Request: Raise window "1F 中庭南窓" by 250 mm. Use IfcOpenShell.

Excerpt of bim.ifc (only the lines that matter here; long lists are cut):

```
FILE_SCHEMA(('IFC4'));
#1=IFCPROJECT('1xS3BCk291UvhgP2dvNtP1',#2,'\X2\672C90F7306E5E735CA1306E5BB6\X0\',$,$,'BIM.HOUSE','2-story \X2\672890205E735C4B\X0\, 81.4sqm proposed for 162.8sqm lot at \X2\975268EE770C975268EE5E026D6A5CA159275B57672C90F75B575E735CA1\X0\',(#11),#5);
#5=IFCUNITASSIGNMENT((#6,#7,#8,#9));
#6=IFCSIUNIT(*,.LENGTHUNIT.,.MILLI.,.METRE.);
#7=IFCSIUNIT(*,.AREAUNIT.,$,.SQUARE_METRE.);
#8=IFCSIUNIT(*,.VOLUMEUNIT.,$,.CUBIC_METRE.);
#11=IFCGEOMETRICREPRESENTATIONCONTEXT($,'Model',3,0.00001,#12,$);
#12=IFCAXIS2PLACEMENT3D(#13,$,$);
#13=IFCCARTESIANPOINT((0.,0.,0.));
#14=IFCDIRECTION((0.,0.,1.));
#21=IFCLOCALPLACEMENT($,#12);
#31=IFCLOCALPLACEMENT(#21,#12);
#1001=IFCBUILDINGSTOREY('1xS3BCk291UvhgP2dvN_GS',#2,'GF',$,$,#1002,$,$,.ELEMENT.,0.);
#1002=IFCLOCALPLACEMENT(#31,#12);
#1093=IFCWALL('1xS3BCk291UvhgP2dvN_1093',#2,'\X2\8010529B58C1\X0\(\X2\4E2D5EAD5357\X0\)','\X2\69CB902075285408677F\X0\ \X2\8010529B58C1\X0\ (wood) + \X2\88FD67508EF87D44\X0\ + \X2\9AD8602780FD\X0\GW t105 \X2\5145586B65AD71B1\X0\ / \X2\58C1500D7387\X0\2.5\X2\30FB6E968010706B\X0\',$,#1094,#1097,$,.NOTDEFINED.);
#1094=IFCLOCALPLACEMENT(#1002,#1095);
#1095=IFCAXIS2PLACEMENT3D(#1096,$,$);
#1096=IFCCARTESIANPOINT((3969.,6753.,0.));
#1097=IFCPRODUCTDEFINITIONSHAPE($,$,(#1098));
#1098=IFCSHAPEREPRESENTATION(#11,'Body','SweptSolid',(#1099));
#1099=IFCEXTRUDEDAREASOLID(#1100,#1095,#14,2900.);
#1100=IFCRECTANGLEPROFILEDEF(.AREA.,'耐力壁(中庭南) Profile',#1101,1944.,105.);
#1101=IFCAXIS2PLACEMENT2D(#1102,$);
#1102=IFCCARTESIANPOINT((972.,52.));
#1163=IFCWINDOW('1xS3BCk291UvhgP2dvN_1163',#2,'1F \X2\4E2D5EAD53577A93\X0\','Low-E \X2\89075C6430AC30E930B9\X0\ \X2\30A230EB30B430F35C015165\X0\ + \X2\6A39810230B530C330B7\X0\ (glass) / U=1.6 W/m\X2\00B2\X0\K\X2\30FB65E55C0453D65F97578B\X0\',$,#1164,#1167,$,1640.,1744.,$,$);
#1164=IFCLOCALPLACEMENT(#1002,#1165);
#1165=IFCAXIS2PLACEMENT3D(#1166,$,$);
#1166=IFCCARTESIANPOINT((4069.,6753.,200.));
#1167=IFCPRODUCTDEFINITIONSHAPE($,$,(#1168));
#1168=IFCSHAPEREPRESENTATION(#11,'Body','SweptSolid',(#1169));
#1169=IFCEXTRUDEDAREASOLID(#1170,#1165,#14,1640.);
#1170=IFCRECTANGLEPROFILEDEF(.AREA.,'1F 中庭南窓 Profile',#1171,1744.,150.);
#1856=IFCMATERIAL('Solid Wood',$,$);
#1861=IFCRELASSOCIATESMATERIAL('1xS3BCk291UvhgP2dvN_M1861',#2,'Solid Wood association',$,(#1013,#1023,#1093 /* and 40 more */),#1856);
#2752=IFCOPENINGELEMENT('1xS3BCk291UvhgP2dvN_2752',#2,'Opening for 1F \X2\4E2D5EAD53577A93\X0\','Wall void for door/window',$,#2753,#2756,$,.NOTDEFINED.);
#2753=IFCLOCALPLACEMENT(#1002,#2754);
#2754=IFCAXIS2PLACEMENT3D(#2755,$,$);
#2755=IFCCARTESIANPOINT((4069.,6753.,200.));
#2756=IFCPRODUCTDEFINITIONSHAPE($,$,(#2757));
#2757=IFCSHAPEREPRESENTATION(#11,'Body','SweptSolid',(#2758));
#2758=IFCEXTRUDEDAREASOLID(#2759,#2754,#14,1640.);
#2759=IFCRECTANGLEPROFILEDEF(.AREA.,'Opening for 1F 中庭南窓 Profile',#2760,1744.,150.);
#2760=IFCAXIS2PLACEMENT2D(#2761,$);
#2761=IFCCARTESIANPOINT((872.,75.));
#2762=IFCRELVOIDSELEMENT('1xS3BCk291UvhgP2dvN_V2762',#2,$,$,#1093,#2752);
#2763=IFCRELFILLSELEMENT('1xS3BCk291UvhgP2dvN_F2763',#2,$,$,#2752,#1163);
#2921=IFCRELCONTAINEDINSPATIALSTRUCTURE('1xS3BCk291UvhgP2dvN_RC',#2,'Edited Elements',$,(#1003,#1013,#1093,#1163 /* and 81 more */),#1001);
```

```python
import numpy as np
import ifcopenshell
import ifcopenshell.api.geometry
import ifcopenshell.util.placement
import ifcopenshell.util.unit

model = ifcopenshell.open("bim.ifc")
unit_scale = ifcopenshell.util.unit.calculate_unit_scale(model)

window = model.by_id(1163)
opening = window.FillsVoids[0].RelatingOpeningElement
dz = 250.0

shift = np.array([0.0, 0.0, dz])
# The window is not placed relative to its opening, so move both.
for product in (opening, window):
    matrix = ifcopenshell.util.placement.get_local_placement(product.ObjectPlacement)
    matrix[:3, 3] += shift
    ifcopenshell.api.geometry.edit_object_placement(model, product=product, matrix=matrix, is_si=False)

print(f"moved by {dz * unit_scale:+.3f} m")

model.write("bim-out.ifc")
```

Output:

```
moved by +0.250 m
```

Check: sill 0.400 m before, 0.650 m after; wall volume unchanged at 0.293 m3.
